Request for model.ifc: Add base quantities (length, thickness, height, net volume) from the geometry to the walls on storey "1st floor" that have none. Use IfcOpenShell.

First a look at what the model holds.

```python
import ifcopenshell
import ifcopenshell.util.element
import ifcopenshell.util.unit

model = ifcopenshell.open("model.ifc")
print(model.schema)
for unit_type in ("LENGTHUNIT", "AREAUNIT", "VOLUMEUNIT"):
    print(unit_type, ifcopenshell.util.unit.calculate_unit_scale(model, unit_type))
storey = next(s for s in model.by_type("IfcBuildingStorey") if s.Name == "1st floor")
walls = [e for e in ifcopenshell.util.element.get_decomposition(storey) if e.is_a("IfcWall")]
for e in sorted(walls, key=lambda e: e.id()):
    print(e.id(), e.is_a(), e.Name, list(ifcopenshell.util.element.get_psets(e, qtos_only=True)), sep=" | ")
```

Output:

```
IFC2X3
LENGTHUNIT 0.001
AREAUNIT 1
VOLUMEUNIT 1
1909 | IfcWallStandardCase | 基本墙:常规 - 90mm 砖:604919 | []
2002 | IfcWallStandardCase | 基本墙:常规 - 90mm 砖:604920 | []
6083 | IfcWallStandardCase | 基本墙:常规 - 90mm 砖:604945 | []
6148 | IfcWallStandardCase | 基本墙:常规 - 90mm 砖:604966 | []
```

```python
import ifcopenshell
import ifcopenshell.api.pset
import ifcopenshell.geom
import ifcopenshell.util.element
import ifcopenshell.util.shape
import ifcopenshell.util.unit

model = ifcopenshell.open("model.ifc")
unit_scale = ifcopenshell.util.unit.calculate_unit_scale(model)
volume_scale = ifcopenshell.util.unit.calculate_unit_scale(model, "VOLUMEUNIT")
settings = ifcopenshell.geom.settings()

storey = next(s for s in model.by_type("IfcBuildingStorey") if s.Name == "1st floor")
walls = [e for e in ifcopenshell.util.element.get_decomposition(storey) if e.is_a("IfcWall")]

for e in sorted(walls, key=lambda e: e.id()):
    if ifcopenshell.util.element.get_psets(e, qtos_only=True, should_inherit=False):
        continue
    # Geometry comes back in metres, in the element's own axes.
    shape = ifcopenshell.geom.create_shape(settings, e)
    values = {
        "Length": ifcopenshell.util.shape.get_x(shape.geometry) / unit_scale,
        "Width": ifcopenshell.util.shape.get_y(shape.geometry) / unit_scale,
        "Height": ifcopenshell.util.shape.get_z(shape.geometry) / unit_scale,
        "NetVolume": ifcopenshell.util.shape.get_volume(shape.geometry) / volume_scale,
    }
    qto = ifcopenshell.api.pset.add_qto(model, product=e, name="BaseQuantities")
    ifcopenshell.api.pset.edit_qto(model, qto=qto, properties=values)
    print(e.id(), {k: round(v, 3) for k, v in values.items()})

model.write("model_rev.ifc")
```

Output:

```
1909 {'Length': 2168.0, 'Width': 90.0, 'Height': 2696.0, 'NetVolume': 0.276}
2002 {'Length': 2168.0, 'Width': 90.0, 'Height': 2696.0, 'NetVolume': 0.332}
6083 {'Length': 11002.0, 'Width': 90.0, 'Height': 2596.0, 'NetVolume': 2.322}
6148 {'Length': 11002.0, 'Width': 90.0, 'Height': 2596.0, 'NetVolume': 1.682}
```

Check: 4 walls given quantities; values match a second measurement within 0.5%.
